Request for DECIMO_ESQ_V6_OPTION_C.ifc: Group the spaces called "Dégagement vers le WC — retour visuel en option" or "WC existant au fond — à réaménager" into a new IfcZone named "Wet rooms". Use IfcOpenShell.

First a look at what the model holds.

```python
import ifcopenshell

model = ifcopenshell.open("DECIMO_ESQ_V6_OPTION_C.ifc")
print(model.schema)
seen = {}
for space in model.by_type("IfcSpace"):
    seen[space.LongName] = seen.get(space.LongName, 0) + 1
for name, count in sorted(seen.items(), key=str):
    print(count, "x", name)
print("zones:", [z.Name for z in model.by_type("IfcZone")][:20])
```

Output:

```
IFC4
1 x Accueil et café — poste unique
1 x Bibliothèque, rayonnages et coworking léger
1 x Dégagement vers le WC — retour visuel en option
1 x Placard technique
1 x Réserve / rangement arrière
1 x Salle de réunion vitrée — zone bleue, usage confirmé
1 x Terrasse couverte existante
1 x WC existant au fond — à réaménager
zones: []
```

```python
import ifcopenshell
import ifcopenshell.api.group
import ifcopenshell.api.root

model = ifcopenshell.open("DECIMO_ESQ_V6_OPTION_C.ifc")

names = {"Dégagement vers le WC — retour visuel en option", "WC existant au fond — à réaménager"}
spaces = [s for s in model.by_type("IfcSpace") if s.LongName in names]

zone = ifcopenshell.api.root.create_entity(model, ifc_class="IfcZone", name="Wet rooms")
ifcopenshell.api.group.assign_group(model, products=spaces, group=zone)
print(len(spaces), "spaces in", zone.Name)

model.write("DECIMO_ESQ_V6_OPTION_C_v2.ifc")
```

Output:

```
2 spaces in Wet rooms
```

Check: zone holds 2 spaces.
